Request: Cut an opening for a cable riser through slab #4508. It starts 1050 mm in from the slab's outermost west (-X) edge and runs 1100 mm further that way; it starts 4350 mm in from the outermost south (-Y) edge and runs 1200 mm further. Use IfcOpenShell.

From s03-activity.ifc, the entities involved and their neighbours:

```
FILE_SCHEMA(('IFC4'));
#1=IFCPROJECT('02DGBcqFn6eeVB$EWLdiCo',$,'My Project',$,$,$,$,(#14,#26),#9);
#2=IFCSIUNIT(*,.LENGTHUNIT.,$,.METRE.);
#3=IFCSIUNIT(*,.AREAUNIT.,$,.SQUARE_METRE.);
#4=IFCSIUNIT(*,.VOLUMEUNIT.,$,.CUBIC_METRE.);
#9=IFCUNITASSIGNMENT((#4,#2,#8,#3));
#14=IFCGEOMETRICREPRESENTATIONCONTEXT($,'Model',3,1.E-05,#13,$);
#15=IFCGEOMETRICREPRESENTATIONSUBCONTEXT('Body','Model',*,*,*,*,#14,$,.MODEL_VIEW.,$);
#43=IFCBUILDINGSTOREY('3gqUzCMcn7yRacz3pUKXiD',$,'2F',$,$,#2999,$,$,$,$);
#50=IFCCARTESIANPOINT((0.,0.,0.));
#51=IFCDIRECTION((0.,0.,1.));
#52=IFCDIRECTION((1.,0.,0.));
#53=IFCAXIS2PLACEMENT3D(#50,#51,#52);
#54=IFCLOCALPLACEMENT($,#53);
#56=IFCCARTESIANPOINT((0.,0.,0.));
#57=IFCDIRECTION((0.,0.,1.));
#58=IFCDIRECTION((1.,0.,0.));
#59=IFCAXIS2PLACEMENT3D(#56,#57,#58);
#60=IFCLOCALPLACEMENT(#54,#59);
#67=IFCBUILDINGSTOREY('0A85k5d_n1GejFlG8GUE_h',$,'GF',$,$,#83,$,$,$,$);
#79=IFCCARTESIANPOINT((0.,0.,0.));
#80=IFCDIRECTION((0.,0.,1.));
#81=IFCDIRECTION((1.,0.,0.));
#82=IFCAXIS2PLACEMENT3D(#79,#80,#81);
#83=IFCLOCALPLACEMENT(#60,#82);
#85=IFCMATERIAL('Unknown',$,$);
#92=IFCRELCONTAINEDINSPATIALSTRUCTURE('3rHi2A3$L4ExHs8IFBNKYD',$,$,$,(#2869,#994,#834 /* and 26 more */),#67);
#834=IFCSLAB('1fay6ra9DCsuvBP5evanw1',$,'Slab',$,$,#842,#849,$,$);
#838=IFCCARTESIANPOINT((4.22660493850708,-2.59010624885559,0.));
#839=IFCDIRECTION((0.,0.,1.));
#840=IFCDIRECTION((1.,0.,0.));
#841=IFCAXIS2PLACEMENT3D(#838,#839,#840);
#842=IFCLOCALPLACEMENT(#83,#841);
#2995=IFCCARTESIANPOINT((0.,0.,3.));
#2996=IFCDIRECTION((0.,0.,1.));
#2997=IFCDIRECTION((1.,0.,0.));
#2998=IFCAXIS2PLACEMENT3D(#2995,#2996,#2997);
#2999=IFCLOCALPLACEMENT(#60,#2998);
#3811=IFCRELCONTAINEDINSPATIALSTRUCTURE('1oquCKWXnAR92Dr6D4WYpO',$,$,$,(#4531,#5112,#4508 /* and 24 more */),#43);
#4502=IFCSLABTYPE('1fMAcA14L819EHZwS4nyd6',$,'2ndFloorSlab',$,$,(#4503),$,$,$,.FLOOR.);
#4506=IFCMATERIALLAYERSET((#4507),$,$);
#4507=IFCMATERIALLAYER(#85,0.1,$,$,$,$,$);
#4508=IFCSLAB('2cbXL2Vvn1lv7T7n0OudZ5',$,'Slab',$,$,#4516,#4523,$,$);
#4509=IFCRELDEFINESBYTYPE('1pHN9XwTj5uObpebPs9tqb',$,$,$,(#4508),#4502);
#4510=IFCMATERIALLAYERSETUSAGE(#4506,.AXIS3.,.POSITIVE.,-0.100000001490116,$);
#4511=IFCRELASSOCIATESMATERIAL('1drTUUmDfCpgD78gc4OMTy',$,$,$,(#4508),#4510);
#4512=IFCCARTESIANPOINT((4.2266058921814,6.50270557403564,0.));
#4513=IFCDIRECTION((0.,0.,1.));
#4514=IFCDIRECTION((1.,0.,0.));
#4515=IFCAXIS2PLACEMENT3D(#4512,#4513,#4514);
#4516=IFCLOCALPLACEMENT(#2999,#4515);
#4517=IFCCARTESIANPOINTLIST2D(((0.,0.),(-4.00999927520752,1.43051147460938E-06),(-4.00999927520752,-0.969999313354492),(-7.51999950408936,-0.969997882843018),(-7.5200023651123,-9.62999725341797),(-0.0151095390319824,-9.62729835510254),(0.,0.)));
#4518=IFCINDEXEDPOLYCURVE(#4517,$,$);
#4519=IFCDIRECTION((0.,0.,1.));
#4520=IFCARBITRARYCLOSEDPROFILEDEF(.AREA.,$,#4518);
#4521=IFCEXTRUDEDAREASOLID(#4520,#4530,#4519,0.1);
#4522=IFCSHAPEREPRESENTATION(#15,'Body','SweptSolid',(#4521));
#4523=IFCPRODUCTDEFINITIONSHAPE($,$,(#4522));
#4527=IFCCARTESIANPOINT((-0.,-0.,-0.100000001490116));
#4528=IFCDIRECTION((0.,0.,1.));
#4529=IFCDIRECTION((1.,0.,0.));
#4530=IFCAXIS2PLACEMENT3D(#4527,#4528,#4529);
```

```python
import numpy as np
import ifcopenshell
import ifcopenshell.api.feature
import ifcopenshell.api.geometry
import ifcopenshell.api.root
import ifcopenshell.geom
import ifcopenshell.util.placement
import ifcopenshell.util.representation
import ifcopenshell.util.shape
import ifcopenshell.util.unit

model = ifcopenshell.open("s03-activity.ifc")
unit_scale = ifcopenshell.util.unit.calculate_unit_scale(model)
settings = ifcopenshell.geom.settings()


def volume(element):
    """Net volume in cubic metres, openings subtracted."""
    shape = ifcopenshell.geom.create_shape(settings, element)
    return ifcopenshell.util.shape.get_volume(shape.geometry)


slab = model.by_guid("2cbXL2Vvn1lv7T7n0OudZ5")
before = volume(slab)

# Extent in the slab's own axes, in metres. The edges named are its -X and -Y sides.
slab_shape = ifcopenshell.geom.create_shape(settings, slab)
vertices = ifcopenshell.util.shape.get_vertices(slab_shape.geometry)
x_min, y_min, bottom = vertices.min(axis=0)
top = vertices[:, 2].max()

opening = ifcopenshell.api.root.create_entity(model, ifc_class="IfcOpeningElement", name="Cable riser opening", predefined_type="OPENING")
context = ifcopenshell.util.representation.get_context(model, "Model", "Body", "MODEL_VIEW")
width, depth = 1.1, 1.2
outline = [(0.0, 0.0), (width, 0.0), (width, depth), (0.0, depth), (0.0, 0.0)]
# Overshoot both faces by 50 mm so the cut is clean.
shape = ifcopenshell.api.geometry.add_slab_representation(
    model, context=context, depth=top - bottom + 0.1, polyline=outline
)
ifcopenshell.api.geometry.assign_representation(model, product=opening, representation=shape)

matrix = ifcopenshell.util.placement.get_local_placement(slab.ObjectPlacement)
matrix[:, 3] = matrix @ np.append(np.array([x_min + 1.05, y_min + 4.35, bottom - 0.05]) / unit_scale, 1.0)
ifcopenshell.api.geometry.edit_object_placement(model, product=opening, matrix=matrix, is_si=False)
ifcopenshell.api.feature.add_feature(model, feature=opening, element=slab)

after = volume(slab)

print(f"slab volume {before:.3f} -> {after:.3f} m3")

model.write("s03-activity_updated.ifc")
```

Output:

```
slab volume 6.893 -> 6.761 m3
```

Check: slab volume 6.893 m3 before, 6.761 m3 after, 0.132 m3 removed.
